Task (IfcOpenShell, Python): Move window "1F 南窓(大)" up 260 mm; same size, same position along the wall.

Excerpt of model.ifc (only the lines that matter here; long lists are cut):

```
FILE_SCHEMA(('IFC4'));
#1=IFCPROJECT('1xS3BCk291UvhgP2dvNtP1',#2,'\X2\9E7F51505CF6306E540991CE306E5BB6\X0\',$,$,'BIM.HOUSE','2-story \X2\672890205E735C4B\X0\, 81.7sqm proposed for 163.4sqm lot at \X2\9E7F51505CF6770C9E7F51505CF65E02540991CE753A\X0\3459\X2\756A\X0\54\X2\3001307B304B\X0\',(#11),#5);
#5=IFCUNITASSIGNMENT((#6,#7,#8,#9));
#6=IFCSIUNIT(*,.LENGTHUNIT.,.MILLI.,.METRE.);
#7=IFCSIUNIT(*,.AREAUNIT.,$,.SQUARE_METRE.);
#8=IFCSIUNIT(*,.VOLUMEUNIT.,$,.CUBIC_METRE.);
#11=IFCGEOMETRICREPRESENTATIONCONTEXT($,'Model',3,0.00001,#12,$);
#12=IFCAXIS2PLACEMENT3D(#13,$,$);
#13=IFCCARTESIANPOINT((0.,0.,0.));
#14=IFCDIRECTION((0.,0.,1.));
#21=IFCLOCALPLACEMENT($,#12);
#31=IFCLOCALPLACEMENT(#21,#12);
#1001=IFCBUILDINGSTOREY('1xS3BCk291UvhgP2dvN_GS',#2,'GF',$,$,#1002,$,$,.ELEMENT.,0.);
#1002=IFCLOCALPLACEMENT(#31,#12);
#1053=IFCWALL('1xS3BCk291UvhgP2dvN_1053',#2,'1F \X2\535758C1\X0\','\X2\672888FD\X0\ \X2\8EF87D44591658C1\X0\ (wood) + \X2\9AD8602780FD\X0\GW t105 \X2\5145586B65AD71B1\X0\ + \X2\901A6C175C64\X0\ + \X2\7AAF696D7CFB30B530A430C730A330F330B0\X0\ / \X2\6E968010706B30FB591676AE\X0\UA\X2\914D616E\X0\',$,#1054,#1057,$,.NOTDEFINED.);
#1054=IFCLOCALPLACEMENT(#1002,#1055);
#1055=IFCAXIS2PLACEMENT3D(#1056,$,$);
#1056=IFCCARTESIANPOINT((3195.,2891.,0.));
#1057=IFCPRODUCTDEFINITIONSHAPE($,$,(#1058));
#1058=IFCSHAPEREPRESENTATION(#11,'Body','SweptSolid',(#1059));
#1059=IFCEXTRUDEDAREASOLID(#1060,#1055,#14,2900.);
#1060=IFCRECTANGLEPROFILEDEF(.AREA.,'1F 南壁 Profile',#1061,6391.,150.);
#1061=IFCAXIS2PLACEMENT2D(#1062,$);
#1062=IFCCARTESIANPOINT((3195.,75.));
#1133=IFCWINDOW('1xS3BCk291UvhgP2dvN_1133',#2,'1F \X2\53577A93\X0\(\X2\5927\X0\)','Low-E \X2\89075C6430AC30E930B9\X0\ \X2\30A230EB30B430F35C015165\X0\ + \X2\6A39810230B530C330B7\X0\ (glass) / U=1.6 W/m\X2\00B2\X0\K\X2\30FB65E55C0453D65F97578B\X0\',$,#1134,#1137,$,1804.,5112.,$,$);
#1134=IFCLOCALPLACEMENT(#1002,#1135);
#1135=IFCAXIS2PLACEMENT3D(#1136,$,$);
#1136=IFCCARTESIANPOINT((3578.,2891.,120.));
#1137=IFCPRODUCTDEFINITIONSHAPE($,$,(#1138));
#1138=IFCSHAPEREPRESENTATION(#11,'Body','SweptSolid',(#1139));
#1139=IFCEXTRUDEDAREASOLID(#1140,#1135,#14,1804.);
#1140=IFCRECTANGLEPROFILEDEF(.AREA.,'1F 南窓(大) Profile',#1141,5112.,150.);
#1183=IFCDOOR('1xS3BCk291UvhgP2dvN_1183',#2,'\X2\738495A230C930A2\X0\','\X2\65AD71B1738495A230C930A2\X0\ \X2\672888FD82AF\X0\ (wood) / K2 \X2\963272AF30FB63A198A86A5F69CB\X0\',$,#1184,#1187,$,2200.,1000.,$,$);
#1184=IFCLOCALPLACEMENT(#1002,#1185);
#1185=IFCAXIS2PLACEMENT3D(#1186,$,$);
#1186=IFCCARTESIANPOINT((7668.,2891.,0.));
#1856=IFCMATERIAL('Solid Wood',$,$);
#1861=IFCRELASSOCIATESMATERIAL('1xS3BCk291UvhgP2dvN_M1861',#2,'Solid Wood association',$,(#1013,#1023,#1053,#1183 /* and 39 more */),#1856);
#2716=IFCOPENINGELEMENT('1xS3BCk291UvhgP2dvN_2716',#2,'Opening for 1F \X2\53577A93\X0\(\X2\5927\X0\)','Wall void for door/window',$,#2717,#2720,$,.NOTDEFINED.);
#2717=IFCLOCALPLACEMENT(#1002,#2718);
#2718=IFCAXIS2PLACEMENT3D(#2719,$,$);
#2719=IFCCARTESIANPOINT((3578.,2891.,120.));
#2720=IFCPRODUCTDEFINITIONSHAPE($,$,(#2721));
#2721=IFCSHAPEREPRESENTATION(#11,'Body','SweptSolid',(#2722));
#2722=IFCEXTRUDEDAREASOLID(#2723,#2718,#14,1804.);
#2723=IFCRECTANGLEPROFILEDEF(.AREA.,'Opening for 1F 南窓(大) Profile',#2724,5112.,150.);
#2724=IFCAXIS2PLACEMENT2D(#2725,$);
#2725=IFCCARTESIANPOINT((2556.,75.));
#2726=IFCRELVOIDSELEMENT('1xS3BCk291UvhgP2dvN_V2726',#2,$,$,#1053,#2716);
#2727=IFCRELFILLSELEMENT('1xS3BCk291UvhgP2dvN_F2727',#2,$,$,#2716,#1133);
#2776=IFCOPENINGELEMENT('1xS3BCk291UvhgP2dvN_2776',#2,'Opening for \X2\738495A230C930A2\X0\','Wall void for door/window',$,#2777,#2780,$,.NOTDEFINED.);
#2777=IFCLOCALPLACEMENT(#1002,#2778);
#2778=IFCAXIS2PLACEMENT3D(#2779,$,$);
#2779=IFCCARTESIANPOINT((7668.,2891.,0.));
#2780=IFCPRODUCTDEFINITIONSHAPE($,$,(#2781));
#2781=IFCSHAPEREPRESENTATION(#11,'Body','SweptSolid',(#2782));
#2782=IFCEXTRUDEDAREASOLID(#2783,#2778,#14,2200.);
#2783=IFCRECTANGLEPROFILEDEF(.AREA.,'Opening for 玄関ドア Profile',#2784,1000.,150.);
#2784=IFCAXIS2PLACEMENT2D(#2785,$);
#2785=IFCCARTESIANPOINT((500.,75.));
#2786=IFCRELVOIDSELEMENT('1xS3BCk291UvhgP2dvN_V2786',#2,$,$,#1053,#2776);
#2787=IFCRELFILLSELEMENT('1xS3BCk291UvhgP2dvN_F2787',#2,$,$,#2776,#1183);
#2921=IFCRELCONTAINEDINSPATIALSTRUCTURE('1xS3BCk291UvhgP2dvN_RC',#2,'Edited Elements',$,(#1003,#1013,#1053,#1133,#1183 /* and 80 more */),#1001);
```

```python
import numpy as np
import ifcopenshell
import ifcopenshell.api.geometry
import ifcopenshell.util.placement
import ifcopenshell.util.unit

model = ifcopenshell.open("model.ifc")
unit_scale = ifcopenshell.util.unit.calculate_unit_scale(model)

window = model.by_id(1133)
opening = window.FillsVoids[0].RelatingOpeningElement
dz = 0.26 / unit_scale

shift = np.array([0.0, 0.0, dz])
# The window is not placed relative to its opening, so move both.
for product in (opening, window):
    matrix = ifcopenshell.util.placement.get_local_placement(product.ObjectPlacement)
    matrix[:3, 3] += shift
    ifcopenshell.api.geometry.edit_object_placement(model, product=product, matrix=matrix, is_si=False)

print(f"moved by {dz * unit_scale:+.3f} m")

model.write("model_edited.ifc")
```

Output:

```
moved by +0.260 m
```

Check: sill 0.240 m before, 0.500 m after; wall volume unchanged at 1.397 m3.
